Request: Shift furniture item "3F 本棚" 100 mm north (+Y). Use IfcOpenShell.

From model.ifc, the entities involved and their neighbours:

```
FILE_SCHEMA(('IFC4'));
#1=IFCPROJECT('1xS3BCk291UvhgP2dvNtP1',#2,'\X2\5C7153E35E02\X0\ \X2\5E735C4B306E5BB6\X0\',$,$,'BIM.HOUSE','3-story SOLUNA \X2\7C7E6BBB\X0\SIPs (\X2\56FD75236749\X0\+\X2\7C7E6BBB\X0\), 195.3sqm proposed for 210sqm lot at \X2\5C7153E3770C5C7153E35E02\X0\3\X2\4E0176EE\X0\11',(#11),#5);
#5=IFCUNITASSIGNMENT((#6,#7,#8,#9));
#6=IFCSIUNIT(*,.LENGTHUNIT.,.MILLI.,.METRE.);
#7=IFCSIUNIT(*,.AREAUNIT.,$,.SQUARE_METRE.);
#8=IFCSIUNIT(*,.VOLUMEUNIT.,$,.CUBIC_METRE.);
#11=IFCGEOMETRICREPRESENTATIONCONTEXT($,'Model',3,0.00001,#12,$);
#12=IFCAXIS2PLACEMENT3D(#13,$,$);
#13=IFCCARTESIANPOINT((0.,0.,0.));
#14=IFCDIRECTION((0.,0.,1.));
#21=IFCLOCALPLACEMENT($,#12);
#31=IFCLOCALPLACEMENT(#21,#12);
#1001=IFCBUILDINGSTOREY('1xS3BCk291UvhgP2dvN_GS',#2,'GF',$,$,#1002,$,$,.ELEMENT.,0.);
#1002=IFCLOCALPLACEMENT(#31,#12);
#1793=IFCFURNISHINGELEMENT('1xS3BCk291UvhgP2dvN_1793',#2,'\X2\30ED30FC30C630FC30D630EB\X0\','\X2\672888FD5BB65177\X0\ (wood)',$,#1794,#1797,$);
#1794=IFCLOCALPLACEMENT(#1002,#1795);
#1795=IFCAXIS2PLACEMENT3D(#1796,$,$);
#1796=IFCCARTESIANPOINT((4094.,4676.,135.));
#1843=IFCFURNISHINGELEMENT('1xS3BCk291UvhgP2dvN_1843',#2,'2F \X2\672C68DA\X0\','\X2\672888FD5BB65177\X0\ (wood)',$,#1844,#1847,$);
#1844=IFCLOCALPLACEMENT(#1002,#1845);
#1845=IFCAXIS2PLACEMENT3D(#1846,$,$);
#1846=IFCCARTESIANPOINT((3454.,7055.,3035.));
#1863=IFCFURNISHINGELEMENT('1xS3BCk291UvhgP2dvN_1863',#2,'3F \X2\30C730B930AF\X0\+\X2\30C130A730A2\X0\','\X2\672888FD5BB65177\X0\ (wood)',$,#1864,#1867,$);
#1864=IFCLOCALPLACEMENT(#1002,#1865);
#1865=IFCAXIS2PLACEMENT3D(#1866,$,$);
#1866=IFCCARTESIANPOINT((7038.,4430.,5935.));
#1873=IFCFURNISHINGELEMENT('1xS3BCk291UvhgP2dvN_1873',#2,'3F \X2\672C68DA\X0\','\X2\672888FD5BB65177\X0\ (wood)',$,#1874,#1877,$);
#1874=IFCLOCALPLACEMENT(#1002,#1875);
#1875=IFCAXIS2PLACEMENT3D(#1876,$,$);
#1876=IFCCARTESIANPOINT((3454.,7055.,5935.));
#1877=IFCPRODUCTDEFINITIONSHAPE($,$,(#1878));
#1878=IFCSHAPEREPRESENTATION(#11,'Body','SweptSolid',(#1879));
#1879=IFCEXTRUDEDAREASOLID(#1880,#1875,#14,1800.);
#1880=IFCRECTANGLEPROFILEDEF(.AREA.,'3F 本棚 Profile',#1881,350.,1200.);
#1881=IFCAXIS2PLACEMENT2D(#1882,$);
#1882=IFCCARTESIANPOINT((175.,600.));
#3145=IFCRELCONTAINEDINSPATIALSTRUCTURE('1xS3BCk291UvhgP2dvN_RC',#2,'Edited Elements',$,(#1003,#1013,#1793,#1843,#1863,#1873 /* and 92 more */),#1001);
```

```python
import ifcopenshell
import ifcopenshell.api.geometry
import ifcopenshell.util.placement
import ifcopenshell.util.unit

model = ifcopenshell.open("model.ifc")
unit_scale = ifcopenshell.util.unit.calculate_unit_scale(model)

item = model.by_id(1873)
matrix = ifcopenshell.util.placement.get_local_placement(item.ObjectPlacement)
matrix[1, 3] += 0.1 / unit_scale
ifcopenshell.api.geometry.edit_object_placement(model, product=item, matrix=matrix, is_si=False)

print(ifcopenshell.util.placement.get_local_placement(item.ObjectPlacement).round(3) + 0.0)

model.write("model_v2.ifc")
```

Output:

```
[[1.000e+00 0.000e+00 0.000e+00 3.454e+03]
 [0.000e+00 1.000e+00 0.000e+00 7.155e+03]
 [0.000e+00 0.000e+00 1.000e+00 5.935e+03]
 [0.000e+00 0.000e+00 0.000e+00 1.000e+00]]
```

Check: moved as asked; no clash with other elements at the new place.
